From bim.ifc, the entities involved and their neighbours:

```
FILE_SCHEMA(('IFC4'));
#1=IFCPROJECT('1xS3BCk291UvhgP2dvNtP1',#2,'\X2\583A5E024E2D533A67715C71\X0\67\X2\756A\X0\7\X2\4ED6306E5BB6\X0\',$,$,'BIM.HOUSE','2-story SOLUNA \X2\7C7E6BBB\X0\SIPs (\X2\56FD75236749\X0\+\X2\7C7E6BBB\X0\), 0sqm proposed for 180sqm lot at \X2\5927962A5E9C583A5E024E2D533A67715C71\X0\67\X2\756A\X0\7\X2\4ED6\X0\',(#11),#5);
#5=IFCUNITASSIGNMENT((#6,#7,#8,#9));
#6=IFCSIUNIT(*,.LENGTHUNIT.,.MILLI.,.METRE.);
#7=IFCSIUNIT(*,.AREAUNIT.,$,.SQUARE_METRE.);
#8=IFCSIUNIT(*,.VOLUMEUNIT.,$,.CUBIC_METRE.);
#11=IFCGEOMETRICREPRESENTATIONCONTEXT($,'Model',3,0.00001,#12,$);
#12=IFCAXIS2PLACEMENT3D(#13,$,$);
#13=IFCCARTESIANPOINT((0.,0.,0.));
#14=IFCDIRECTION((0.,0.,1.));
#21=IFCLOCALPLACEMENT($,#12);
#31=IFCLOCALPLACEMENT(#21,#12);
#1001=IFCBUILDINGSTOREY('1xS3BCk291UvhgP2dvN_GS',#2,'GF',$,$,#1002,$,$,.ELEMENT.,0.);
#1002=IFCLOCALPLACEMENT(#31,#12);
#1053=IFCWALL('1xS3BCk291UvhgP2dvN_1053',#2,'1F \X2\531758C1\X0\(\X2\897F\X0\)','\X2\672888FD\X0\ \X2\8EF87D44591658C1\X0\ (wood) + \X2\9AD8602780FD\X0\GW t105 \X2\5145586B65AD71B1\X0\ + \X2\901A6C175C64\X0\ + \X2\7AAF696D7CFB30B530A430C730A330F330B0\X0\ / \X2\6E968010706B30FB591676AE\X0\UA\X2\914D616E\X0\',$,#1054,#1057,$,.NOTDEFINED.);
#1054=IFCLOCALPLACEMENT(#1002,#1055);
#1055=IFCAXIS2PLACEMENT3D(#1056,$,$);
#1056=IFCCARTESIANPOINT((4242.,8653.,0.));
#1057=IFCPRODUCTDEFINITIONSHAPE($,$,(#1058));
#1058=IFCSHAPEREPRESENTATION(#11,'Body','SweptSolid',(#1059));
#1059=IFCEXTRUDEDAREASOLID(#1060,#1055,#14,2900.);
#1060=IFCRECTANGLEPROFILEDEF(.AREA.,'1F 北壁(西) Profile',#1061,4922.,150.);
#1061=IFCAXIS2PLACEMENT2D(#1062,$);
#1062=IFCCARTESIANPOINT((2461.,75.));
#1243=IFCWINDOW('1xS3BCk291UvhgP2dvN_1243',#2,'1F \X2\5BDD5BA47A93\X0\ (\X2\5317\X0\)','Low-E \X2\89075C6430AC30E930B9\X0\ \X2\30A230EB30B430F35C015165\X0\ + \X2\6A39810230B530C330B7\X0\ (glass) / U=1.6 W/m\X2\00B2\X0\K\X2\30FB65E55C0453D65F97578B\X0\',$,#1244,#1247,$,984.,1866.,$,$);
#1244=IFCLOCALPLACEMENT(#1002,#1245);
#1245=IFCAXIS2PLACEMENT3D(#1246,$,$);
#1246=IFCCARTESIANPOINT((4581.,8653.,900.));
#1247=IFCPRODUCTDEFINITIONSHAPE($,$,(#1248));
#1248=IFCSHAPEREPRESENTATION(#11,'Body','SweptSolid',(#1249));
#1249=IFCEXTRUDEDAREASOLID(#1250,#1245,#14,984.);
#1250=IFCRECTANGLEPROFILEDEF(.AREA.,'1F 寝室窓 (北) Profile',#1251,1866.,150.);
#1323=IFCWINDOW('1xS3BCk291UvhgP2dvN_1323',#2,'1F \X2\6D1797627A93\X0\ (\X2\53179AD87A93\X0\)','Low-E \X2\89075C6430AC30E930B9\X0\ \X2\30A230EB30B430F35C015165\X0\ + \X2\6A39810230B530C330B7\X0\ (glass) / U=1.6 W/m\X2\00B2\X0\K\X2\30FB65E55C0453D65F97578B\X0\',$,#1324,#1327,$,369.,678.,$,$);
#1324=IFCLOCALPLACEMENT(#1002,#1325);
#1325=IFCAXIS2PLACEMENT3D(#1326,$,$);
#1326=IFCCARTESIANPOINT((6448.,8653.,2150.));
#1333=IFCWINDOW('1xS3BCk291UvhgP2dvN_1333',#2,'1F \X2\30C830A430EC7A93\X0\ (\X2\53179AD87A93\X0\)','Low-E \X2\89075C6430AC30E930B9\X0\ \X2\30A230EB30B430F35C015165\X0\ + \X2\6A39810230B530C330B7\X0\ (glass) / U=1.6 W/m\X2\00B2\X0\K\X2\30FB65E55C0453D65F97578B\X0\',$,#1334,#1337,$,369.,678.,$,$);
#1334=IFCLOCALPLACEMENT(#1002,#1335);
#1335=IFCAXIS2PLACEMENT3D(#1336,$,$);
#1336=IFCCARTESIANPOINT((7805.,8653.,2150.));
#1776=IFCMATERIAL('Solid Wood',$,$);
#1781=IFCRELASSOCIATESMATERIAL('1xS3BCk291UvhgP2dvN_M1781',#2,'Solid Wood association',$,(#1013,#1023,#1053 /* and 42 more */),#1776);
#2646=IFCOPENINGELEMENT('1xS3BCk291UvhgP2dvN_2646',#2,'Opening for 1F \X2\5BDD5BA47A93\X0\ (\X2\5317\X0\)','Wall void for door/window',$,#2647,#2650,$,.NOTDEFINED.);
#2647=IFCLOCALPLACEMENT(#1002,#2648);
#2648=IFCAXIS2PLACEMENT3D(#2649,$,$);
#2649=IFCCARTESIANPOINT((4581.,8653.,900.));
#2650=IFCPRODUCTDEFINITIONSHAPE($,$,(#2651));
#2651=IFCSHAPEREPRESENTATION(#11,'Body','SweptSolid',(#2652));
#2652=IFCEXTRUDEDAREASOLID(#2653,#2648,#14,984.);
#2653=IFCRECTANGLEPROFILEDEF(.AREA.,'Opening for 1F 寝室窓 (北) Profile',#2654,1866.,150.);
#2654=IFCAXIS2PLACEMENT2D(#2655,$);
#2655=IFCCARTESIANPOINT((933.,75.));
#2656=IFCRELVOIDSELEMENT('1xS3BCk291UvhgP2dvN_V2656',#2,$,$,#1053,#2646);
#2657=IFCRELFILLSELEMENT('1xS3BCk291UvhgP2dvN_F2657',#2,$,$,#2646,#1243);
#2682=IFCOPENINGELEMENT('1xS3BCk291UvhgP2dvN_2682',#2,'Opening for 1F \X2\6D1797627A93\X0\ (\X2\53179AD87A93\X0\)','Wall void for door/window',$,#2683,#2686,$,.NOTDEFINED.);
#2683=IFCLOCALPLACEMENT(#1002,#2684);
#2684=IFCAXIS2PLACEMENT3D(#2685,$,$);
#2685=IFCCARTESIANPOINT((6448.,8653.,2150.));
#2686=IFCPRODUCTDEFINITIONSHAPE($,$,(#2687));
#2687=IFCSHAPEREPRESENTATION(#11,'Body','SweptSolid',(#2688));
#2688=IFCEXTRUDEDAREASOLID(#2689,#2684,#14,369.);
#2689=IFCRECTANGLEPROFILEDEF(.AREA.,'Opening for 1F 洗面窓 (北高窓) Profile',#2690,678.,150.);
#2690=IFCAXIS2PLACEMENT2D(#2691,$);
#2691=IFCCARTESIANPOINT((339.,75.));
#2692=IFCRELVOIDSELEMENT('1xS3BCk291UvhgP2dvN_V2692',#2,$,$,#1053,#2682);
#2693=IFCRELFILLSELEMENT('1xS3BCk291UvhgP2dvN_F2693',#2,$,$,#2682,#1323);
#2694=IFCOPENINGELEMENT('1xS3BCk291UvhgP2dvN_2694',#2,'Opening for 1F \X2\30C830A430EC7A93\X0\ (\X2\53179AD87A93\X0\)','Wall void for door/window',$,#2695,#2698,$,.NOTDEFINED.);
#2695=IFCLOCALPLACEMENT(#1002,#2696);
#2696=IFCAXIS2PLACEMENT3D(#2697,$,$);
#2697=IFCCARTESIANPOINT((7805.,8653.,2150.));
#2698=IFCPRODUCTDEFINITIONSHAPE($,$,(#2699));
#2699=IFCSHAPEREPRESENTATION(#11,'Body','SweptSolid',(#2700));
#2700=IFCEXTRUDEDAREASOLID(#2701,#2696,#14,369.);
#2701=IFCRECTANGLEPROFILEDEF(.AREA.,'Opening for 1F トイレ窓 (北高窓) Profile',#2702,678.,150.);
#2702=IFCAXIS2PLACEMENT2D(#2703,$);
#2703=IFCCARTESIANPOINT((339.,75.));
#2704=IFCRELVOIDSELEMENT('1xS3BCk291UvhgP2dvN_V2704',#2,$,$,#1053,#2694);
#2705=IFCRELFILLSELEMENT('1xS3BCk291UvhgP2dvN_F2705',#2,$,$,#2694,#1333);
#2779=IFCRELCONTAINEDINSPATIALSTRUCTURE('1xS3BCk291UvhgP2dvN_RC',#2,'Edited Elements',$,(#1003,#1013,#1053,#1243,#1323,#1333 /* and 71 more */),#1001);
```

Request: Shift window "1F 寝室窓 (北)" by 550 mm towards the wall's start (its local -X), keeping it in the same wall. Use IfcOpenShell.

```python
import ifcopenshell
import ifcopenshell.api.geometry
import ifcopenshell.util.placement
import ifcopenshell.util.unit

model = ifcopenshell.open("bim.ifc")
unit_scale = ifcopenshell.util.unit.calculate_unit_scale(model)

window = model.by_guid("1xS3BCk291UvhgP2dvN_1243")
opening = window.FillsVoids[0].RelatingOpeningElement
wall = opening.VoidsElements[0].RelatingBuildingElement

wall_matrix = ifcopenshell.util.placement.get_local_placement(wall.ObjectPlacement)
shift = wall_matrix[:3, 0] * -0.55 / unit_scale
before = ifcopenshell.util.placement.get_local_placement(window.ObjectPlacement)[:3, 3].copy()

# The window is not placed relative to its opening, so move both.
for product in (opening, window):
    matrix = ifcopenshell.util.placement.get_local_placement(product.ObjectPlacement)
    matrix[:3, 3] += shift
    ifcopenshell.api.geometry.edit_object_placement(model, product=product, matrix=matrix, is_si=False)

after = ifcopenshell.util.placement.get_local_placement(window.ObjectPlacement)[:3, 3]
print("window moved by", (after - before).round(3) + 0.0)

model.write("bim_v2.ifc")
```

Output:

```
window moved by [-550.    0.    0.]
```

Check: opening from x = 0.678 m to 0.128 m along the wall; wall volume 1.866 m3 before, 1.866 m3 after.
